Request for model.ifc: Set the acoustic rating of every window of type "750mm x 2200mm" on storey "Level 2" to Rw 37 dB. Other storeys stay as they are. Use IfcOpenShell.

First a look at what the model holds.

```python
import ifcopenshell
import ifcopenshell.util.element

model = ifcopenshell.open("model.ifc")
print(model.schema)
storey = next(s for s in model.by_type("IfcBuildingStorey") if s.Name == "Level 2")
windows = [e for e in ifcopenshell.util.element.get_decomposition(storey) if e.is_a("IfcWindow")]
seen = {}
for e in windows:
    element_type = ifcopenshell.util.element.get_type(e)
    key = (element_type.Name if element_type != e and element_type else None, ifcopenshell.util.element.get_pset(e, "Pset_WindowCommon", "AcousticRating"))
    seen[key] = seen.get(key, 0) + 1
for (name, value), count in sorted(seen.items(), key=str):
    print(count, "x", name, "|", value)
```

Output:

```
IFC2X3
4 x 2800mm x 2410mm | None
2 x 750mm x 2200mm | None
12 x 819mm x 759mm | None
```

```python
import ifcopenshell
import ifcopenshell.api.pset
import ifcopenshell.util.element

model = ifcopenshell.open("model.ifc")

storey = next(s for s in model.by_type("IfcBuildingStorey") if s.Name == "Level 2")
windows = [e for e in ifcopenshell.util.element.get_decomposition(storey) if e.is_a("IfcWindow")]

count = 0
for e in windows:
    element_type = ifcopenshell.util.element.get_type(e)
    if element_type in (None, e) or element_type.Name != "750mm x 2200mm":
        continue
    # add_pset returns the element's existing set when there is one.
    pset = ifcopenshell.api.pset.add_pset(model, product=e, name="Pset_WindowCommon")
    ifcopenshell.api.pset.edit_pset(model, pset=pset, properties={"AcousticRating": "Rw 37 dB"})
    count += 1

print(count, "windows updated")

model.write("model_updated.ifc")
```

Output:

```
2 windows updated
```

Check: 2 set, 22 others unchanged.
